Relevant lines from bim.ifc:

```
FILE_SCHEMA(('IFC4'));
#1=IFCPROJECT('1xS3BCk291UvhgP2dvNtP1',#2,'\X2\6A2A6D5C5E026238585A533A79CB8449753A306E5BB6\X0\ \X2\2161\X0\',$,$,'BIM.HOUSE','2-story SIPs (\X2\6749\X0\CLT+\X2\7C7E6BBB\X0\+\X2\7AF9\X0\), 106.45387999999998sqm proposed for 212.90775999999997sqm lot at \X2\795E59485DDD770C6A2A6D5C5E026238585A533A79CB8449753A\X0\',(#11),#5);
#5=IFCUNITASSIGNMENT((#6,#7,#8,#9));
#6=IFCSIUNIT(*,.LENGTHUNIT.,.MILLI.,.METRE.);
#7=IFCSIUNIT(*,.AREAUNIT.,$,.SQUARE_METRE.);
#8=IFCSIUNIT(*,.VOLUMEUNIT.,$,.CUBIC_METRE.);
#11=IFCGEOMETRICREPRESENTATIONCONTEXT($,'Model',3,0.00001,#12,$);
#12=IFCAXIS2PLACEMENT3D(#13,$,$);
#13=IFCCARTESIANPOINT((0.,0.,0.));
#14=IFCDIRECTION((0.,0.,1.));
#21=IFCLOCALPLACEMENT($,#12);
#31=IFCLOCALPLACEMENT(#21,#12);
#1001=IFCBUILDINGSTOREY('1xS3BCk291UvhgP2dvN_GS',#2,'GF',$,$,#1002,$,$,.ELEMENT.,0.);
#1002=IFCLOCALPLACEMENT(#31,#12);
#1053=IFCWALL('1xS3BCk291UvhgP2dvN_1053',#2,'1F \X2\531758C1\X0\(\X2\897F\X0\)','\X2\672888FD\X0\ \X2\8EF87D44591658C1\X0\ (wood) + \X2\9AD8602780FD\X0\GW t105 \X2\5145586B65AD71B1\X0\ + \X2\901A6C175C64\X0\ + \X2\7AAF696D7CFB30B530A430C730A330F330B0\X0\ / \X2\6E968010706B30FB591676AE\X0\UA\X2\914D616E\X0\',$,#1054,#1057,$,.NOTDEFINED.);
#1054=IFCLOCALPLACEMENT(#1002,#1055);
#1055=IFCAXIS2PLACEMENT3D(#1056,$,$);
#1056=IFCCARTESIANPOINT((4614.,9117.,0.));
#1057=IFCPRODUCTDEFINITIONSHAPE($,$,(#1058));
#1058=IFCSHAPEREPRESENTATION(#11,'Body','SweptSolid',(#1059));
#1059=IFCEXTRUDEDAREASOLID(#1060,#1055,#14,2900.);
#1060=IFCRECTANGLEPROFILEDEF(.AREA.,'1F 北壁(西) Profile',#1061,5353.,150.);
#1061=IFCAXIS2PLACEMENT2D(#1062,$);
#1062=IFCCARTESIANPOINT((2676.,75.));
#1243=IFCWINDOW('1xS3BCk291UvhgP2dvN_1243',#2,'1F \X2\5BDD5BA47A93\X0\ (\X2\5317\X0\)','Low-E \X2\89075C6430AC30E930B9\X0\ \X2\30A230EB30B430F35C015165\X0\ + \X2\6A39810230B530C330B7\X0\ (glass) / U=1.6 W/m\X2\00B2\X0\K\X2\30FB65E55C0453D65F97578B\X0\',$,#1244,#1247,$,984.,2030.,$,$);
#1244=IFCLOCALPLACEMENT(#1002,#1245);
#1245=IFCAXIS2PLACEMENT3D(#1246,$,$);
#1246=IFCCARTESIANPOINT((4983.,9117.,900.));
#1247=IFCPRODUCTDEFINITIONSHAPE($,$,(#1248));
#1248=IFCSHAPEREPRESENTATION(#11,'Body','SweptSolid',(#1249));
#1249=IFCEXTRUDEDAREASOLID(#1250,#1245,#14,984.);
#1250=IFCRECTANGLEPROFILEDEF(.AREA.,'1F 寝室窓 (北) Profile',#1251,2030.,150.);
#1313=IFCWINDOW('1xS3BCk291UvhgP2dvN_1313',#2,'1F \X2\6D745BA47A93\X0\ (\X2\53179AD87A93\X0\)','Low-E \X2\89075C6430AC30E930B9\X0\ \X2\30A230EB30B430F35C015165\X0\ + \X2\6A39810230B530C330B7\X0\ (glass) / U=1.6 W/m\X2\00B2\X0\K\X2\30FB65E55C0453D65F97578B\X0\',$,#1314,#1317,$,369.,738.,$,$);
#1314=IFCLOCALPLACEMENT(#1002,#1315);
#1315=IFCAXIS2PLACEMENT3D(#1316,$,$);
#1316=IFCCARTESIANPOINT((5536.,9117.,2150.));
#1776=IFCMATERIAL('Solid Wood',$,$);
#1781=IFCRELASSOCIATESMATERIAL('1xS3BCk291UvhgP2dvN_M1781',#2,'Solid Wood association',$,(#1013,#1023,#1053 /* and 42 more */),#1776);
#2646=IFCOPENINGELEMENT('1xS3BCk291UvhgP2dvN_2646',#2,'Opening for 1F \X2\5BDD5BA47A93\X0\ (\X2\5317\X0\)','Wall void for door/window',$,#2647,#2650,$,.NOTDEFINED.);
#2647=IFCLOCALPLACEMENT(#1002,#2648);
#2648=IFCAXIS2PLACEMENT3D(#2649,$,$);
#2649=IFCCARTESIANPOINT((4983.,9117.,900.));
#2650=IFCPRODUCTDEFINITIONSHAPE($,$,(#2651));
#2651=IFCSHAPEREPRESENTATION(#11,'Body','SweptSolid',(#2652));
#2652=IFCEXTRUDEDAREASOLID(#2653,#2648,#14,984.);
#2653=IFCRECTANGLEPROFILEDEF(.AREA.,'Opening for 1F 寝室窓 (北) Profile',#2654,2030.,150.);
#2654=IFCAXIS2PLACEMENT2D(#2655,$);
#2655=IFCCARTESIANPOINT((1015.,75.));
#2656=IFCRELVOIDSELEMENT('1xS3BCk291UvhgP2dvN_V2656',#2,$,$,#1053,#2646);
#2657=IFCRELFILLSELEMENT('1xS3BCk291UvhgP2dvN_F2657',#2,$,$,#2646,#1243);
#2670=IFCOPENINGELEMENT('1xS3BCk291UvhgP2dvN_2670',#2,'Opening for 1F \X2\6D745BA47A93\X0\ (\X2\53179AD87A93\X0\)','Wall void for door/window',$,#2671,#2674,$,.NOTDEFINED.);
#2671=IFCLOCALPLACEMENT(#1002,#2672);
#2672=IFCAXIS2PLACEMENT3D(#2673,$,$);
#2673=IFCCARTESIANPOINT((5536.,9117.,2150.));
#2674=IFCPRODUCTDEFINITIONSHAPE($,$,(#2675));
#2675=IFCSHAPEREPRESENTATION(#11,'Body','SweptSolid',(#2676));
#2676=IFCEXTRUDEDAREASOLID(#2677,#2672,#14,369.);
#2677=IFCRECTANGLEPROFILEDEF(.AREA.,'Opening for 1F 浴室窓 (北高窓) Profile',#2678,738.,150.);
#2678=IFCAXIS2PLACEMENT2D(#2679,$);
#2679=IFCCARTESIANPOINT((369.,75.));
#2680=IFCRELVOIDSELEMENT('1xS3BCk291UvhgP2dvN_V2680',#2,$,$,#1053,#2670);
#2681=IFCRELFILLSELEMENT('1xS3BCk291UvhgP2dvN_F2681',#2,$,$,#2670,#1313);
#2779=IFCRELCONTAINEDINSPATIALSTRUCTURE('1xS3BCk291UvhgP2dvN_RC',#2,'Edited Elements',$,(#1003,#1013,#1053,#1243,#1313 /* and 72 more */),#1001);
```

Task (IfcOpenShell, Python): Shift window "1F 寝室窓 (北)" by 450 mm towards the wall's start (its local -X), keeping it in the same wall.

```python
import ifcopenshell
import ifcopenshell.api.geometry
import ifcopenshell.util.placement

model = ifcopenshell.open("bim.ifc")

window = model.by_id(1243)
opening = window.FillsVoids[0].RelatingOpeningElement
wall = opening.VoidsElements[0].RelatingBuildingElement

wall_matrix = ifcopenshell.util.placement.get_local_placement(wall.ObjectPlacement)
shift = wall_matrix[:3, 0] * -450.0
before = ifcopenshell.util.placement.get_local_placement(window.ObjectPlacement)[:3, 3].copy()

# The window is not placed relative to its opening, so move both.
for product in (opening, window):
    matrix = ifcopenshell.util.placement.get_local_placement(product.ObjectPlacement)
    matrix[:3, 3] += shift
    ifcopenshell.api.geometry.edit_object_placement(model, product=product, matrix=matrix, is_si=False)

after = ifcopenshell.util.placement.get_local_placement(window.ObjectPlacement)[:3, 3]
print("window moved by", (after - before).round(3) + 0.0)

model.write("bim_rev.ifc")
```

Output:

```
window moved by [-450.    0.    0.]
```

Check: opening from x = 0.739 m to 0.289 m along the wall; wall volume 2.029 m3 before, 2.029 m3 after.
